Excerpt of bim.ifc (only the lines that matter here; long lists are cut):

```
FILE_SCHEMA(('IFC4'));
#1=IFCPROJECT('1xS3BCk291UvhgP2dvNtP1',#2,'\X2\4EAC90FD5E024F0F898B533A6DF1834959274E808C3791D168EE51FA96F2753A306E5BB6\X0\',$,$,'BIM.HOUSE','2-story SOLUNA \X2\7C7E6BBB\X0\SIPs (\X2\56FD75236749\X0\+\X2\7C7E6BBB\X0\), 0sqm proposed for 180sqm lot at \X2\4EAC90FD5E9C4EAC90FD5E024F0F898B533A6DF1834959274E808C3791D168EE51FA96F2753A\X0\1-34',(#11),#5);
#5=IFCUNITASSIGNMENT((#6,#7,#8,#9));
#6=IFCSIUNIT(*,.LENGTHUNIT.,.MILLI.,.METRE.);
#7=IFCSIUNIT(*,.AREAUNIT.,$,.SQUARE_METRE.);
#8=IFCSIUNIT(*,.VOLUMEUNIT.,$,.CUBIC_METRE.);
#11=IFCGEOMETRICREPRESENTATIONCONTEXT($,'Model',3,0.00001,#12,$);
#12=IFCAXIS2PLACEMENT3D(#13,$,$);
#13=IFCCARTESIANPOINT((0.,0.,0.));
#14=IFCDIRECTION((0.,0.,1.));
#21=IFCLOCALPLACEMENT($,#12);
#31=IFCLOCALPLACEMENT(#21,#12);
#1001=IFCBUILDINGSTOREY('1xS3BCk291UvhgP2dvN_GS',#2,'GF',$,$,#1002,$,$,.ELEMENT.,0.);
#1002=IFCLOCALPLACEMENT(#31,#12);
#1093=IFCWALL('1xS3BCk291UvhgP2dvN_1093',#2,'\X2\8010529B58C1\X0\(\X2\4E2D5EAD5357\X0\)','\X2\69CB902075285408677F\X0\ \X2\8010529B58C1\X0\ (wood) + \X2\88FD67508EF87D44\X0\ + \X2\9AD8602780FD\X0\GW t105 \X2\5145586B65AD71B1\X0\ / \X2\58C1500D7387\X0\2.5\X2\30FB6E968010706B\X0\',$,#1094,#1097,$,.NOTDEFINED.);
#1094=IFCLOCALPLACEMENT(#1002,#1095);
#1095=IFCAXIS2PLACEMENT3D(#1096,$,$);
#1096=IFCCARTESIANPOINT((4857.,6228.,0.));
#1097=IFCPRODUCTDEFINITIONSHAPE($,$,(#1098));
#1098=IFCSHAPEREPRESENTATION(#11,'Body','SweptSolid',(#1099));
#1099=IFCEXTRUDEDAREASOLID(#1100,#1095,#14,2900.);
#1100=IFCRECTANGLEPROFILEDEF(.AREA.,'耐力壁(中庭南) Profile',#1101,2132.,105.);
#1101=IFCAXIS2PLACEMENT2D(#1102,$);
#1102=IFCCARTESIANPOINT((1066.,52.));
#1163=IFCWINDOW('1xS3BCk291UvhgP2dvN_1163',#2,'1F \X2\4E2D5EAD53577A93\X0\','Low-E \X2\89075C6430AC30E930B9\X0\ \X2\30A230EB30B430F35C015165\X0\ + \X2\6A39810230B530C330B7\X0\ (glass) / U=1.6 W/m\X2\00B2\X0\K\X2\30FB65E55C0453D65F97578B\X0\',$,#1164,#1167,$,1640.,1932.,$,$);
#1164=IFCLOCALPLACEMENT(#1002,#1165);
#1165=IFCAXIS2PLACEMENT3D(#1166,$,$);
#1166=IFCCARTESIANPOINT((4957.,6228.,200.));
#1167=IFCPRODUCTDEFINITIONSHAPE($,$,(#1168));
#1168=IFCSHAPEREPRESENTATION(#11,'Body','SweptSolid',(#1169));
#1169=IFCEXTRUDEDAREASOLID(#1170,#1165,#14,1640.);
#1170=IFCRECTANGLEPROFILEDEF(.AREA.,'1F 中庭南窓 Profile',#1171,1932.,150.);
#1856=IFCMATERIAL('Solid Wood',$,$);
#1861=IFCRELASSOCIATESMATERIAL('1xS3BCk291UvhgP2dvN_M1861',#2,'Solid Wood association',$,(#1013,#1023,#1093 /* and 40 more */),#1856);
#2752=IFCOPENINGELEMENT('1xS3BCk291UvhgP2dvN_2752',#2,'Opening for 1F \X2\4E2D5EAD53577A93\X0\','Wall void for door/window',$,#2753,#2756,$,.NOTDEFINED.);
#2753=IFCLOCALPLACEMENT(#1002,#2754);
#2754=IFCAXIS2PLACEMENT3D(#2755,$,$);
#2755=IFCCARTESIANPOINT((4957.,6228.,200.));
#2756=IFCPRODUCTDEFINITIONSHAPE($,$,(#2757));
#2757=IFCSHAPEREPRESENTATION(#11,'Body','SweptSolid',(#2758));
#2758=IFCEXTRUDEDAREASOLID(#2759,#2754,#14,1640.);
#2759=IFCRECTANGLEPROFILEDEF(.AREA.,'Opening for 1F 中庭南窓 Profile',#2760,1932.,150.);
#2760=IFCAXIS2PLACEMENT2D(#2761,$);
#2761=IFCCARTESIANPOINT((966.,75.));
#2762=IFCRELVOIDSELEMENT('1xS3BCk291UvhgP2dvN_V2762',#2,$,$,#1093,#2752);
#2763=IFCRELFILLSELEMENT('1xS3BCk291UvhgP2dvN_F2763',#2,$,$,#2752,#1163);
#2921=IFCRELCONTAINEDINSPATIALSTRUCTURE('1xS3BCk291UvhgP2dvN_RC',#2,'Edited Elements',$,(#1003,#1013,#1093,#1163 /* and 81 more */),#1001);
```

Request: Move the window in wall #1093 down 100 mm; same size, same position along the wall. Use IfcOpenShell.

```python
import numpy as np
import ifcopenshell
import ifcopenshell.api.geometry
import ifcopenshell.util.placement
import ifcopenshell.util.unit

model = ifcopenshell.open("bim.ifc")
unit_scale = ifcopenshell.util.unit.calculate_unit_scale(model)

window = model.by_guid("1xS3BCk291UvhgP2dvN_1163")
opening = window.FillsVoids[0].RelatingOpeningElement
dz = -0.1 / unit_scale

shift = np.array([0.0, 0.0, dz])
# The window is not placed relative to its opening, so move both.
for product in (opening, window):
    matrix = ifcopenshell.util.placement.get_local_placement(product.ObjectPlacement)
    matrix[:3, 3] += shift
    ifcopenshell.api.geometry.edit_object_placement(model, product=product, matrix=matrix, is_si=False)

print(f"moved by {dz * unit_scale:+.3f} m")

model.write("bim_v2.ifc")
```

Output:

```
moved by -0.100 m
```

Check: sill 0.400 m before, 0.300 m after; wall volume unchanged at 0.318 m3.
